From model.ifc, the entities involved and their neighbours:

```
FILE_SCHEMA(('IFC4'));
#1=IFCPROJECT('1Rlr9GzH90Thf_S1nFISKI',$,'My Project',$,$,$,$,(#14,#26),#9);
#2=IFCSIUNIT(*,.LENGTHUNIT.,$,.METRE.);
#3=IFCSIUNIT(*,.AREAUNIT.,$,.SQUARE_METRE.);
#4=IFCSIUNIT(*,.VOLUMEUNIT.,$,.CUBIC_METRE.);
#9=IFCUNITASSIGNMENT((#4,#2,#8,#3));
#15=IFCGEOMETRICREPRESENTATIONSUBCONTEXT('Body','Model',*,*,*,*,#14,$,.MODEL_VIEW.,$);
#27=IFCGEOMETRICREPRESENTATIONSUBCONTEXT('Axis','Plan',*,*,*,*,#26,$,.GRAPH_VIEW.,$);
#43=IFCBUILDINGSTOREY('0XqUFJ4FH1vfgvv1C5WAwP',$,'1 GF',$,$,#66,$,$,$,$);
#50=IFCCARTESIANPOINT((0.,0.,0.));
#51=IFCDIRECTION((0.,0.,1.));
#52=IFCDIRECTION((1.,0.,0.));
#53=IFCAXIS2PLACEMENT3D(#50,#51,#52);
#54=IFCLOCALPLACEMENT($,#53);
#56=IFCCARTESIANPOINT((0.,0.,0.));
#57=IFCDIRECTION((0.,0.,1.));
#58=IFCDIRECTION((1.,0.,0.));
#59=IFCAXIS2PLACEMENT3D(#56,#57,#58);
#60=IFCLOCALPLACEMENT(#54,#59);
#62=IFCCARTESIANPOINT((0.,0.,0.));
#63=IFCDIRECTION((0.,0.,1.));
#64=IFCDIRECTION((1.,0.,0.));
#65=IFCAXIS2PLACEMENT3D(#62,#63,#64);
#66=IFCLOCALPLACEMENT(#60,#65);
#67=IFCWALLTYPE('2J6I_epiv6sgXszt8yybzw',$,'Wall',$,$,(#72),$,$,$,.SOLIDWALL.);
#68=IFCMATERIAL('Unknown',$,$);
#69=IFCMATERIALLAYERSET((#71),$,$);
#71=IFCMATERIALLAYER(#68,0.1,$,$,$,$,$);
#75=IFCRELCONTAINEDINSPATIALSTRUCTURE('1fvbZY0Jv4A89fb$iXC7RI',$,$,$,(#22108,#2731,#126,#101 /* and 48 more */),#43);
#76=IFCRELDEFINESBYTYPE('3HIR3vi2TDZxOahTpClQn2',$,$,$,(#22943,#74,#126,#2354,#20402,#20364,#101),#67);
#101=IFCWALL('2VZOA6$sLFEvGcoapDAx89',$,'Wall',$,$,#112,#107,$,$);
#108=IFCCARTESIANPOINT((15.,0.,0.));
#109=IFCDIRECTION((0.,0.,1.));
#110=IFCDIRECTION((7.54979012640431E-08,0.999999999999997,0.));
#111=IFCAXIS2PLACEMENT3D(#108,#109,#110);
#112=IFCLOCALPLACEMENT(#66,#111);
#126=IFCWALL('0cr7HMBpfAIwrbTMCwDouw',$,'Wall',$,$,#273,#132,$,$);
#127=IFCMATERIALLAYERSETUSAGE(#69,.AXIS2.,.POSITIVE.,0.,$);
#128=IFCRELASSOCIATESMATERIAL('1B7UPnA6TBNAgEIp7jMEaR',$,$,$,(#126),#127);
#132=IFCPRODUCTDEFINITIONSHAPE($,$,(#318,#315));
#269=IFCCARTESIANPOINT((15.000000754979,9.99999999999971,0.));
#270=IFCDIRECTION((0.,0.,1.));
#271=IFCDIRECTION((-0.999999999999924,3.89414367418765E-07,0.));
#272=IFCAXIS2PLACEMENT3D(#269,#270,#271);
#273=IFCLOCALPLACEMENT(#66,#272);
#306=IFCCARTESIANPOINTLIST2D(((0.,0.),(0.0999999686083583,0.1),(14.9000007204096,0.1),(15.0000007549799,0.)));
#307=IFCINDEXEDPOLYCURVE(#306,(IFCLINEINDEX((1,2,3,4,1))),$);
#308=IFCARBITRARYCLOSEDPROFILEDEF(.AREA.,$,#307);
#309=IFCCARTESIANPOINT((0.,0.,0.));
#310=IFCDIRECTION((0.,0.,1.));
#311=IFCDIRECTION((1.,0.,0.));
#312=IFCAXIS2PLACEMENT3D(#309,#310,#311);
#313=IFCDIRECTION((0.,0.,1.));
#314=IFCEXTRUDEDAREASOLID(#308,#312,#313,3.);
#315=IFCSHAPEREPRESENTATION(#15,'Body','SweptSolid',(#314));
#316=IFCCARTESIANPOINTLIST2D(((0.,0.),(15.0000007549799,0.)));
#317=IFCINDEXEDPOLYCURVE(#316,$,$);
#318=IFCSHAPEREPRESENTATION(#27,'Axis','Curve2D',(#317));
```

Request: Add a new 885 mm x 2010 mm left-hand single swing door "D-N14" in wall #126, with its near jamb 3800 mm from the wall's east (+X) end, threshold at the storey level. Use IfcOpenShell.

```python
import numpy as np
import ifcopenshell
import ifcopenshell.api.feature
import ifcopenshell.api.geometry
import ifcopenshell.api.root
import ifcopenshell.api.spatial
import ifcopenshell.geom
import ifcopenshell.util.element
import ifcopenshell.util.placement
import ifcopenshell.util.representation
import ifcopenshell.util.shape
import ifcopenshell.util.unit

model = ifcopenshell.open("model.ifc")
unit_scale = ifcopenshell.util.unit.calculate_unit_scale(model)
settings = ifcopenshell.geom.settings()


def volume(element):
    """Net volume in cubic metres, openings subtracted."""
    shape = ifcopenshell.geom.create_shape(settings, element)
    return ifcopenshell.util.shape.get_volume(shape.geometry)


wall = model.by_guid("0cr7HMBpfAIwrbTMCwDouw")
storey = ifcopenshell.util.element.get_container(wall, ifc_class="IfcBuildingStorey")
context = ifcopenshell.util.representation.get_context(model, "Model", "Body", "MODEL_VIEW")
before = volume(wall)

width, height, from_end, sill = 0.885, 2.01, 3.8, 0.0  # metres

# The wall runs along its own X axis, and the end named is its -X end.
wall_shape = ifcopenshell.geom.create_shape(settings, wall)
x, y, z = ifcopenshell.util.shape.get_vertices(wall_shape.geometry).T
start = x.min() + from_end
face, thickness = float(y.min()), float(y.max() - y.min())
wall_matrix = ifcopenshell.util.placement.get_local_placement(wall.ObjectPlacement)
level = ifcopenshell.util.placement.get_local_placement(storey.ObjectPlacement)[2, 3]


def in_wall(x, y):
    """Placement at x, y metres in the wall's axes, at sill height."""
    matrix = wall_matrix.copy()
    matrix[:, 3] = wall_matrix @ np.array([x / unit_scale, y / unit_scale, 0.0, 1.0])
    matrix[2, 3] = level + sill / unit_scale
    return matrix


# Opening: a box that overshoots both wall faces by 50 mm.
opening = ifcopenshell.api.root.create_entity(model, ifc_class="IfcOpeningElement", predefined_type="OPENING")
box = ifcopenshell.api.geometry.add_wall_representation(
    model, context=context, length=width, height=height, thickness=thickness + 0.1
)
ifcopenshell.api.geometry.assign_representation(model, product=opening, representation=box)
ifcopenshell.api.geometry.edit_object_placement(model, product=opening, matrix=in_wall(start, face - 0.05), is_si=False)
ifcopenshell.api.feature.add_feature(model, feature=opening, element=wall)

door = ifcopenshell.api.root.create_entity(model, ifc_class="IfcDoor", name="D-N14", predefined_type="DOOR")
door.OverallWidth, door.OverallHeight = width / unit_scale, height / unit_scale
door.OperationType = "SINGLE_SWING_LEFT"
body = ifcopenshell.api.geometry.add_door_representation(
    model,
    context=context,
    overall_width=door.OverallWidth,
    overall_height=door.OverallHeight,
    operation_type="SINGLE_SWING_LEFT",
    lining_properties={"LiningDepth": thickness / unit_scale, "ThresholdDepth": thickness / unit_scale},
)
ifcopenshell.api.geometry.assign_representation(model, product=door, representation=body)
ifcopenshell.api.spatial.assign_container(model, products=[door], relating_structure=storey)
ifcopenshell.api.feature.add_filling(model, opening=opening, element=door)

# The lining spans the wall, so the door starts at the wall face.
ifcopenshell.api.geometry.edit_object_placement(model, product=door, matrix=in_wall(start, face), is_si=False)

after = volume(wall)

print(f"wall volume {before:.3f} -> {after:.3f} m3")

model.write("model_v2.ifc")
```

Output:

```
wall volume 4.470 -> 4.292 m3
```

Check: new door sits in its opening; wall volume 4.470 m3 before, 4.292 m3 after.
